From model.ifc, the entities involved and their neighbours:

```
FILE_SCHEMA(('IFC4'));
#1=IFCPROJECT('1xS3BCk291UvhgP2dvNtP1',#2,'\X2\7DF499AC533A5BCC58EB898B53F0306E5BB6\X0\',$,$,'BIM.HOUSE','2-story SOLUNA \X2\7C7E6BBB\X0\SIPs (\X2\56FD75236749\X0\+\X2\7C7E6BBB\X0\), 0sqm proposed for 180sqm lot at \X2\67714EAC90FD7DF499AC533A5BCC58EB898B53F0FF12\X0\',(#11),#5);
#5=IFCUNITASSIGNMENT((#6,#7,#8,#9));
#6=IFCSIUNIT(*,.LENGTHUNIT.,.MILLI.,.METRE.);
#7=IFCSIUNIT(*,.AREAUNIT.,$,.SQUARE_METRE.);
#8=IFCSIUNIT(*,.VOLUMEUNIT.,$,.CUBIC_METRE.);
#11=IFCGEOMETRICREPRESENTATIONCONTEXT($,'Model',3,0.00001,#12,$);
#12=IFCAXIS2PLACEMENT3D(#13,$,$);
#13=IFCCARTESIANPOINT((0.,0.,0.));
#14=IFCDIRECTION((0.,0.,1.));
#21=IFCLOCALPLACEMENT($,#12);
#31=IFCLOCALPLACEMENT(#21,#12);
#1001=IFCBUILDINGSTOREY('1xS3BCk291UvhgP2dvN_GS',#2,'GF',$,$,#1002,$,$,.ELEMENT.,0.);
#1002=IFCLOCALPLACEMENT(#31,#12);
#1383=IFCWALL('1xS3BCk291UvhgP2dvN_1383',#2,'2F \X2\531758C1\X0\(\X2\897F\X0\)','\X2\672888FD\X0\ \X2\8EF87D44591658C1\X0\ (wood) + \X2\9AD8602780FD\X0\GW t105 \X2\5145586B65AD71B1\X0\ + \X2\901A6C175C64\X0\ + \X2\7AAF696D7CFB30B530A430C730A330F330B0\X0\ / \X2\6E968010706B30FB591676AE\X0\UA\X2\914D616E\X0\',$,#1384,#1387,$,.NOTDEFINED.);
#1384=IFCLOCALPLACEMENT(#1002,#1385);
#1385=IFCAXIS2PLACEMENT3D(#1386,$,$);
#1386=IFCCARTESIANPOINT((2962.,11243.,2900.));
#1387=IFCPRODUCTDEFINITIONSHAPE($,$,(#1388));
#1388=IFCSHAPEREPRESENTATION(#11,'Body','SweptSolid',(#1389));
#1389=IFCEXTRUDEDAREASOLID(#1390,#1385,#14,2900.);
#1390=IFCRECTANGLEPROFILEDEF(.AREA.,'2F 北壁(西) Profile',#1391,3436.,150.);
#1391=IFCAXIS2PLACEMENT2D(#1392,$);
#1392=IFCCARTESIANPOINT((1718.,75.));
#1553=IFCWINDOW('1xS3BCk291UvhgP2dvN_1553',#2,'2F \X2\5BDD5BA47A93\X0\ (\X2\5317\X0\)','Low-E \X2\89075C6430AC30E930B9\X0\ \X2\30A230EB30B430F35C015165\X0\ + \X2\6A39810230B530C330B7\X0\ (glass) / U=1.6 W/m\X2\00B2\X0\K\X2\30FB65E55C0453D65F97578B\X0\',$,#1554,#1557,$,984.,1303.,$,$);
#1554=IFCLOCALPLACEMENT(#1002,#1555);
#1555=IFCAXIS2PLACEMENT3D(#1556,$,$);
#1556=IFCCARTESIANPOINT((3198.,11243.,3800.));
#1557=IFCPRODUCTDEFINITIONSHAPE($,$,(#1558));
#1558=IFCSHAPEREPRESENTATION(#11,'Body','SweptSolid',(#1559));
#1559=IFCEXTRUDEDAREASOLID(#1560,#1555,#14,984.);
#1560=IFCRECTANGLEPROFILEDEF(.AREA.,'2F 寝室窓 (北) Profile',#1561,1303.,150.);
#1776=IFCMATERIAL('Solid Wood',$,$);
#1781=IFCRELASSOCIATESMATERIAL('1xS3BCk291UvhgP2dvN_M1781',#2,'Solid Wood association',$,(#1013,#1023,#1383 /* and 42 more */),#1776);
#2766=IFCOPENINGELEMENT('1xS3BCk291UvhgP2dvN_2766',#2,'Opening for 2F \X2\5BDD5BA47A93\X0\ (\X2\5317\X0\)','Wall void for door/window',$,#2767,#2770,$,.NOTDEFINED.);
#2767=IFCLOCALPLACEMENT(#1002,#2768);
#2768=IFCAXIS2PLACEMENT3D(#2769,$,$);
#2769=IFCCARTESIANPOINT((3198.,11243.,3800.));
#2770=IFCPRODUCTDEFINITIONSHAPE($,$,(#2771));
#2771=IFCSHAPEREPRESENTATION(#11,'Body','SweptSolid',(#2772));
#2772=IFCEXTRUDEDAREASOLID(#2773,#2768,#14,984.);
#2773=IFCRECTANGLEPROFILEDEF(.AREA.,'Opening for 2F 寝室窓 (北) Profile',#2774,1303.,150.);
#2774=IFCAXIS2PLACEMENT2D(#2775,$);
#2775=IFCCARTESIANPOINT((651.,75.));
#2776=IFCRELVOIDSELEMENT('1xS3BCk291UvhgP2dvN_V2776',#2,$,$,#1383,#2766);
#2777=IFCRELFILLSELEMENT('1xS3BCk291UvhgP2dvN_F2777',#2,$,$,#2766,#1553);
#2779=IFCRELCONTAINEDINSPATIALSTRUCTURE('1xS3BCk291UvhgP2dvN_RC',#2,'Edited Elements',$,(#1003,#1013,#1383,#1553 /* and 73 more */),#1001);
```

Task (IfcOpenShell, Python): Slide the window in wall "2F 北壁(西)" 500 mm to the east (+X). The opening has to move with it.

```python
import ifcopenshell
import ifcopenshell.api.geometry
import ifcopenshell.util.placement
import ifcopenshell.util.unit

model = ifcopenshell.open("model.ifc")
unit_scale = ifcopenshell.util.unit.calculate_unit_scale(model)

window = model.by_guid("1xS3BCk291UvhgP2dvN_1553")
opening = window.FillsVoids[0].RelatingOpeningElement
wall = opening.VoidsElements[0].RelatingBuildingElement

wall_matrix = ifcopenshell.util.placement.get_local_placement(wall.ObjectPlacement)
shift = wall_matrix[:3, 0] * 0.5 / unit_scale
before = ifcopenshell.util.placement.get_local_placement(window.ObjectPlacement)[:3, 3].copy()

# The window is not placed relative to its opening, so move both.
for product in (opening, window):
    matrix = ifcopenshell.util.placement.get_local_placement(product.ObjectPlacement)
    matrix[:3, 3] += shift
    ifcopenshell.api.geometry.edit_object_placement(model, product=product, matrix=matrix, is_si=False)

after = ifcopenshell.util.placement.get_local_placement(window.ObjectPlacement)[:3, 3]
print("window moved by", (after - before).round(3) + 0.0)

model.write("model_updated.ifc")
```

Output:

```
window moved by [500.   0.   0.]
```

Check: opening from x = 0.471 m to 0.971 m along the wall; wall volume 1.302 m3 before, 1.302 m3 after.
